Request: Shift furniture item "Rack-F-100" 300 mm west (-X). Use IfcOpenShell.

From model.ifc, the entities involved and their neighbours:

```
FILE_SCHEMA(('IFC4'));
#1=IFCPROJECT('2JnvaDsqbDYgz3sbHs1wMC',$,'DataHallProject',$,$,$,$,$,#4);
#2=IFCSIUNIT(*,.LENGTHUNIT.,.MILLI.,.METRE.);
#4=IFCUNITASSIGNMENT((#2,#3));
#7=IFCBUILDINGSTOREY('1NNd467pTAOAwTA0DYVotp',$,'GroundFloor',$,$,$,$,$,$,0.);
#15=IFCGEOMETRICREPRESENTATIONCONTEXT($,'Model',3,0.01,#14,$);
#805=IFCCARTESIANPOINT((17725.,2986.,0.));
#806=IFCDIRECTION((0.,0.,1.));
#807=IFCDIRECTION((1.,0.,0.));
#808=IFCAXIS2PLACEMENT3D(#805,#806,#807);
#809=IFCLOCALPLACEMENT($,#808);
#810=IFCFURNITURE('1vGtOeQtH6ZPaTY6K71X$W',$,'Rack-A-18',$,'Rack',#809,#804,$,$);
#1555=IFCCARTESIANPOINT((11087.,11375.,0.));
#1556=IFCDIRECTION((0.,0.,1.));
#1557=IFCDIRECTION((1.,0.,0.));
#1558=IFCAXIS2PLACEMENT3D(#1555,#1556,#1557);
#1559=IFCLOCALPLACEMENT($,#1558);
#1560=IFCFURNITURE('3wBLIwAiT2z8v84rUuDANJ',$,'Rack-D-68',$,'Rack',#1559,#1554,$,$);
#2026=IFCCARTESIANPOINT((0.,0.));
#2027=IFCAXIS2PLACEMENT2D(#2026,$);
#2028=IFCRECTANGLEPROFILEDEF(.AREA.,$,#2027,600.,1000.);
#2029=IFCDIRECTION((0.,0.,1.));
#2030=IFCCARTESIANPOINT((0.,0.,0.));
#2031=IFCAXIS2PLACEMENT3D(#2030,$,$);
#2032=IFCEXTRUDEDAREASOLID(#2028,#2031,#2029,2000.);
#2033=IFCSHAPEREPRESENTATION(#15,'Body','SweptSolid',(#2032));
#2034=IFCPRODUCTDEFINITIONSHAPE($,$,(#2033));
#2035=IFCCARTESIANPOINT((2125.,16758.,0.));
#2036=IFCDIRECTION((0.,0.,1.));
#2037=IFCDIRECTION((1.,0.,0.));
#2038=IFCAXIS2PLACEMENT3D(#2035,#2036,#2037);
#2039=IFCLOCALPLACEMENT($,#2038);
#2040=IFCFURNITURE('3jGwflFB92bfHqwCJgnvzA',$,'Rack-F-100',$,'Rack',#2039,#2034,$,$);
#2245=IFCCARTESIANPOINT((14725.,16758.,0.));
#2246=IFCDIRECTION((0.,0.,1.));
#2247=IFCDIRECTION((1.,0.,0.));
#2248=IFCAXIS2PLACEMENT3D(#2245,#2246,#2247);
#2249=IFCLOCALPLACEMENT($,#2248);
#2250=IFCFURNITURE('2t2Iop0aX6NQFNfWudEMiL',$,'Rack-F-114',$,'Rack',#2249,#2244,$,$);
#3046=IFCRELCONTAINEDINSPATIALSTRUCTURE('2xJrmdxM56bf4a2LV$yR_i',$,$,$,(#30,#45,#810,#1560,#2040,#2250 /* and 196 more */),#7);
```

```python
import ifcopenshell
import ifcopenshell.api.geometry
import ifcopenshell.util.placement

model = ifcopenshell.open("model.ifc")

item = model.by_guid("3jGwflFB92bfHqwCJgnvzA")
matrix = ifcopenshell.util.placement.get_local_placement(item.ObjectPlacement)
matrix[0, 3] -= 300.0
ifcopenshell.api.geometry.edit_object_placement(model, product=item, matrix=matrix, is_si=False)

print(ifcopenshell.util.placement.get_local_placement(item.ObjectPlacement).round(3) + 0.0)

model.write("model_v2.ifc")
```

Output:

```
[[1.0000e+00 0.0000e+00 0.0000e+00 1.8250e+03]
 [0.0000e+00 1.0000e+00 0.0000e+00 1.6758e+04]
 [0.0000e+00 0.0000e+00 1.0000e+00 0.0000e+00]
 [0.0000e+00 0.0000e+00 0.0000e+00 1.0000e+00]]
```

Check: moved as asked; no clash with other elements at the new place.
